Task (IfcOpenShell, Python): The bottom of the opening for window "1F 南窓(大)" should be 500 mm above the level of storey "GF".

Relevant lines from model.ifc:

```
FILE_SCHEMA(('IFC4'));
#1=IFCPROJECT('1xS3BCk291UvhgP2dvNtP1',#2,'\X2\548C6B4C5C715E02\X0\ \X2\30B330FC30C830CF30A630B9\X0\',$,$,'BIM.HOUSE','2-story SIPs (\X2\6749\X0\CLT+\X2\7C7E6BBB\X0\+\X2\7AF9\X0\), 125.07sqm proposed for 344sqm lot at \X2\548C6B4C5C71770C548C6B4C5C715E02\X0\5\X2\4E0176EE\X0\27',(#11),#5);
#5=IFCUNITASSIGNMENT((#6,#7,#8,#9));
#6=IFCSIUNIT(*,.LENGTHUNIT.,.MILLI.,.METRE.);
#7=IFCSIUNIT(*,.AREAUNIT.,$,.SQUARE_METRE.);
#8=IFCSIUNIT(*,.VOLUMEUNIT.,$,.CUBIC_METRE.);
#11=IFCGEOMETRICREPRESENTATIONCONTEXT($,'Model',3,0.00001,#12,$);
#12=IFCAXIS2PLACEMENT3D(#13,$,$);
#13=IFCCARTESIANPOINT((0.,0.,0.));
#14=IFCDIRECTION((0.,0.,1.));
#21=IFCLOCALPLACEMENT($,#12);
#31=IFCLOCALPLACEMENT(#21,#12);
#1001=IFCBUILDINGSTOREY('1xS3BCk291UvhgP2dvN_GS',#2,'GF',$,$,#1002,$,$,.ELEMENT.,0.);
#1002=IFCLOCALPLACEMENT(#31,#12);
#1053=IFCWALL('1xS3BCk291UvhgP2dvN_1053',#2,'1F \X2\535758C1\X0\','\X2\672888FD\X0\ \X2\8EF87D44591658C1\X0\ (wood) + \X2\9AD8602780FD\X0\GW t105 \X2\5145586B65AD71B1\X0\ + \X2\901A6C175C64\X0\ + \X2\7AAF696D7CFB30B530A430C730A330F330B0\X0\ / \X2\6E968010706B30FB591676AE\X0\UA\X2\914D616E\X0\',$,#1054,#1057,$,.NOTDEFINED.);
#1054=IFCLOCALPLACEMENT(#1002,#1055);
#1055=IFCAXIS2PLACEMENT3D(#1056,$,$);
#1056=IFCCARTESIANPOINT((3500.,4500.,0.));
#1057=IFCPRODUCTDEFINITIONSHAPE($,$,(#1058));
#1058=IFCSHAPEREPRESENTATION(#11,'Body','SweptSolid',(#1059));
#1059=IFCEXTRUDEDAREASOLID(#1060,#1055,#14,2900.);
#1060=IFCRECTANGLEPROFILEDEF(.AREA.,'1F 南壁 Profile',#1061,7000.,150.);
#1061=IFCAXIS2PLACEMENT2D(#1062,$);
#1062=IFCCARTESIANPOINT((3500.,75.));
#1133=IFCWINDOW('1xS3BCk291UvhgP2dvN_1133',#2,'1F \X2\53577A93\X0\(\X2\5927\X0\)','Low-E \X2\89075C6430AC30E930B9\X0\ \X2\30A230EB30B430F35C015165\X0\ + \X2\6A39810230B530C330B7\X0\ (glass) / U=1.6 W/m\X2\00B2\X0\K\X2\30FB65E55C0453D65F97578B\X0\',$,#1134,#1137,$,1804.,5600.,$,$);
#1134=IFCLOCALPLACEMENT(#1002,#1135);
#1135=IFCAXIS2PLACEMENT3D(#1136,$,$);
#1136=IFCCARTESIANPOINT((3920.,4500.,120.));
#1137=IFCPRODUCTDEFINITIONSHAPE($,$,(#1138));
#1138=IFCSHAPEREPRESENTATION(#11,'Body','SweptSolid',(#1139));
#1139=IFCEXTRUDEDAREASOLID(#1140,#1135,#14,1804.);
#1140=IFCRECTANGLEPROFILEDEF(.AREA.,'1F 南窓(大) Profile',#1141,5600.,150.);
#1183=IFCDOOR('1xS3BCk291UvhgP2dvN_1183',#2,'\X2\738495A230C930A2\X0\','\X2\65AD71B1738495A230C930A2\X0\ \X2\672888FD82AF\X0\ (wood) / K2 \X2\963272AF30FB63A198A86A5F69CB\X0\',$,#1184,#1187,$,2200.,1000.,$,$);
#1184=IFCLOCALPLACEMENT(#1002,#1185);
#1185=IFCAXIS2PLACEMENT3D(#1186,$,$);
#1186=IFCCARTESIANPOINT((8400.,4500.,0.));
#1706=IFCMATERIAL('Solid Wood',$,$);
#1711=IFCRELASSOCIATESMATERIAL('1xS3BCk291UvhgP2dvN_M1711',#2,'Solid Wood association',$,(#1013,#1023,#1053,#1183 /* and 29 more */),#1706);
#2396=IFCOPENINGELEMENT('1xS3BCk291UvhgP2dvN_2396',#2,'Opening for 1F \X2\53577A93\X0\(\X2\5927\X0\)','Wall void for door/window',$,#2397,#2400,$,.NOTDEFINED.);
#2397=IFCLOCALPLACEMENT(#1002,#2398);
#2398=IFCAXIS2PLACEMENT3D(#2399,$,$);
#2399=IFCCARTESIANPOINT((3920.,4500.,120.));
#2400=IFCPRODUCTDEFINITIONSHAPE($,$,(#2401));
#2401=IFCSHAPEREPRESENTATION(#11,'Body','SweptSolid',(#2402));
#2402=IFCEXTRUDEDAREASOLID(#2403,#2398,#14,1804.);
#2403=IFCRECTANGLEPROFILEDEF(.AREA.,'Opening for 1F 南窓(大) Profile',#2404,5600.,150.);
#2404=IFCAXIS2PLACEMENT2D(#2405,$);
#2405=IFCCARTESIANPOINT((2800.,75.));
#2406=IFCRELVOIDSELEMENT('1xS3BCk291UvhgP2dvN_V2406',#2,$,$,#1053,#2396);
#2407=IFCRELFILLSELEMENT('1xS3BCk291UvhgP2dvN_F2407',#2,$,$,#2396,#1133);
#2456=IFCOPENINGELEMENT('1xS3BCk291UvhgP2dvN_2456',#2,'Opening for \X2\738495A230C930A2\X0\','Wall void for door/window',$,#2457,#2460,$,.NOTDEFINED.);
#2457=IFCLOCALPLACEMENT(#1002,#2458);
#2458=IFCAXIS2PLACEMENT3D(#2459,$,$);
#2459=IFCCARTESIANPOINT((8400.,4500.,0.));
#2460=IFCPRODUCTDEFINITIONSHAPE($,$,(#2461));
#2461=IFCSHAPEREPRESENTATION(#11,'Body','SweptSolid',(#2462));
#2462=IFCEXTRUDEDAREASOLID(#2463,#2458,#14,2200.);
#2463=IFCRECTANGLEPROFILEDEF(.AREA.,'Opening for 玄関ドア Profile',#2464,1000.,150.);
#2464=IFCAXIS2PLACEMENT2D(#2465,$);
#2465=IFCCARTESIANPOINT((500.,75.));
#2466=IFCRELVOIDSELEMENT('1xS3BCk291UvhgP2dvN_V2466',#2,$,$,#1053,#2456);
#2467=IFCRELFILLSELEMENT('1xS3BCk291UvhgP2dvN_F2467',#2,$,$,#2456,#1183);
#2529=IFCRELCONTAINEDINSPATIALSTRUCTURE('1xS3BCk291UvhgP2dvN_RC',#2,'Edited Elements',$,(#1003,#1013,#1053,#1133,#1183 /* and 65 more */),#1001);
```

```python
import numpy as np
import ifcopenshell
import ifcopenshell.api.geometry
import ifcopenshell.geom
import ifcopenshell.util.element
import ifcopenshell.util.placement
import ifcopenshell.util.shape
import ifcopenshell.util.unit

model = ifcopenshell.open("model.ifc")
unit_scale = ifcopenshell.util.unit.calculate_unit_scale(model)

window = model.by_guid("1xS3BCk291UvhgP2dvN_1133")
opening = window.FillsVoids[0].RelatingOpeningElement
storey = ifcopenshell.util.element.get_container(window, ifc_class="IfcBuildingStorey")
level = ifcopenshell.util.placement.get_local_placement(storey.ObjectPlacement)[2, 3]

# The opening's origin need not be at the sill, so measure its lowest point.
shape = ifcopenshell.geom.create_shape(ifcopenshell.geom.settings(), opening)
bottom = ifcopenshell.util.shape.get_shape_bottom_elevation(shape, shape.geometry) / unit_scale
dz = level + 0.5 / unit_scale - bottom

shift = np.array([0.0, 0.0, dz])
# The window is not placed relative to its opening, so move both.
for product in (opening, window):
    matrix = ifcopenshell.util.placement.get_local_placement(product.ObjectPlacement)
    matrix[:3, 3] += shift
    ifcopenshell.api.geometry.edit_object_placement(model, product=product, matrix=matrix, is_si=False)

print(f"moved by {dz * unit_scale:+.3f} m")

model.write("model_v2.ifc")
```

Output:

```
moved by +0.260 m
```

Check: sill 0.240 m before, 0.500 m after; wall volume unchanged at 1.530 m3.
